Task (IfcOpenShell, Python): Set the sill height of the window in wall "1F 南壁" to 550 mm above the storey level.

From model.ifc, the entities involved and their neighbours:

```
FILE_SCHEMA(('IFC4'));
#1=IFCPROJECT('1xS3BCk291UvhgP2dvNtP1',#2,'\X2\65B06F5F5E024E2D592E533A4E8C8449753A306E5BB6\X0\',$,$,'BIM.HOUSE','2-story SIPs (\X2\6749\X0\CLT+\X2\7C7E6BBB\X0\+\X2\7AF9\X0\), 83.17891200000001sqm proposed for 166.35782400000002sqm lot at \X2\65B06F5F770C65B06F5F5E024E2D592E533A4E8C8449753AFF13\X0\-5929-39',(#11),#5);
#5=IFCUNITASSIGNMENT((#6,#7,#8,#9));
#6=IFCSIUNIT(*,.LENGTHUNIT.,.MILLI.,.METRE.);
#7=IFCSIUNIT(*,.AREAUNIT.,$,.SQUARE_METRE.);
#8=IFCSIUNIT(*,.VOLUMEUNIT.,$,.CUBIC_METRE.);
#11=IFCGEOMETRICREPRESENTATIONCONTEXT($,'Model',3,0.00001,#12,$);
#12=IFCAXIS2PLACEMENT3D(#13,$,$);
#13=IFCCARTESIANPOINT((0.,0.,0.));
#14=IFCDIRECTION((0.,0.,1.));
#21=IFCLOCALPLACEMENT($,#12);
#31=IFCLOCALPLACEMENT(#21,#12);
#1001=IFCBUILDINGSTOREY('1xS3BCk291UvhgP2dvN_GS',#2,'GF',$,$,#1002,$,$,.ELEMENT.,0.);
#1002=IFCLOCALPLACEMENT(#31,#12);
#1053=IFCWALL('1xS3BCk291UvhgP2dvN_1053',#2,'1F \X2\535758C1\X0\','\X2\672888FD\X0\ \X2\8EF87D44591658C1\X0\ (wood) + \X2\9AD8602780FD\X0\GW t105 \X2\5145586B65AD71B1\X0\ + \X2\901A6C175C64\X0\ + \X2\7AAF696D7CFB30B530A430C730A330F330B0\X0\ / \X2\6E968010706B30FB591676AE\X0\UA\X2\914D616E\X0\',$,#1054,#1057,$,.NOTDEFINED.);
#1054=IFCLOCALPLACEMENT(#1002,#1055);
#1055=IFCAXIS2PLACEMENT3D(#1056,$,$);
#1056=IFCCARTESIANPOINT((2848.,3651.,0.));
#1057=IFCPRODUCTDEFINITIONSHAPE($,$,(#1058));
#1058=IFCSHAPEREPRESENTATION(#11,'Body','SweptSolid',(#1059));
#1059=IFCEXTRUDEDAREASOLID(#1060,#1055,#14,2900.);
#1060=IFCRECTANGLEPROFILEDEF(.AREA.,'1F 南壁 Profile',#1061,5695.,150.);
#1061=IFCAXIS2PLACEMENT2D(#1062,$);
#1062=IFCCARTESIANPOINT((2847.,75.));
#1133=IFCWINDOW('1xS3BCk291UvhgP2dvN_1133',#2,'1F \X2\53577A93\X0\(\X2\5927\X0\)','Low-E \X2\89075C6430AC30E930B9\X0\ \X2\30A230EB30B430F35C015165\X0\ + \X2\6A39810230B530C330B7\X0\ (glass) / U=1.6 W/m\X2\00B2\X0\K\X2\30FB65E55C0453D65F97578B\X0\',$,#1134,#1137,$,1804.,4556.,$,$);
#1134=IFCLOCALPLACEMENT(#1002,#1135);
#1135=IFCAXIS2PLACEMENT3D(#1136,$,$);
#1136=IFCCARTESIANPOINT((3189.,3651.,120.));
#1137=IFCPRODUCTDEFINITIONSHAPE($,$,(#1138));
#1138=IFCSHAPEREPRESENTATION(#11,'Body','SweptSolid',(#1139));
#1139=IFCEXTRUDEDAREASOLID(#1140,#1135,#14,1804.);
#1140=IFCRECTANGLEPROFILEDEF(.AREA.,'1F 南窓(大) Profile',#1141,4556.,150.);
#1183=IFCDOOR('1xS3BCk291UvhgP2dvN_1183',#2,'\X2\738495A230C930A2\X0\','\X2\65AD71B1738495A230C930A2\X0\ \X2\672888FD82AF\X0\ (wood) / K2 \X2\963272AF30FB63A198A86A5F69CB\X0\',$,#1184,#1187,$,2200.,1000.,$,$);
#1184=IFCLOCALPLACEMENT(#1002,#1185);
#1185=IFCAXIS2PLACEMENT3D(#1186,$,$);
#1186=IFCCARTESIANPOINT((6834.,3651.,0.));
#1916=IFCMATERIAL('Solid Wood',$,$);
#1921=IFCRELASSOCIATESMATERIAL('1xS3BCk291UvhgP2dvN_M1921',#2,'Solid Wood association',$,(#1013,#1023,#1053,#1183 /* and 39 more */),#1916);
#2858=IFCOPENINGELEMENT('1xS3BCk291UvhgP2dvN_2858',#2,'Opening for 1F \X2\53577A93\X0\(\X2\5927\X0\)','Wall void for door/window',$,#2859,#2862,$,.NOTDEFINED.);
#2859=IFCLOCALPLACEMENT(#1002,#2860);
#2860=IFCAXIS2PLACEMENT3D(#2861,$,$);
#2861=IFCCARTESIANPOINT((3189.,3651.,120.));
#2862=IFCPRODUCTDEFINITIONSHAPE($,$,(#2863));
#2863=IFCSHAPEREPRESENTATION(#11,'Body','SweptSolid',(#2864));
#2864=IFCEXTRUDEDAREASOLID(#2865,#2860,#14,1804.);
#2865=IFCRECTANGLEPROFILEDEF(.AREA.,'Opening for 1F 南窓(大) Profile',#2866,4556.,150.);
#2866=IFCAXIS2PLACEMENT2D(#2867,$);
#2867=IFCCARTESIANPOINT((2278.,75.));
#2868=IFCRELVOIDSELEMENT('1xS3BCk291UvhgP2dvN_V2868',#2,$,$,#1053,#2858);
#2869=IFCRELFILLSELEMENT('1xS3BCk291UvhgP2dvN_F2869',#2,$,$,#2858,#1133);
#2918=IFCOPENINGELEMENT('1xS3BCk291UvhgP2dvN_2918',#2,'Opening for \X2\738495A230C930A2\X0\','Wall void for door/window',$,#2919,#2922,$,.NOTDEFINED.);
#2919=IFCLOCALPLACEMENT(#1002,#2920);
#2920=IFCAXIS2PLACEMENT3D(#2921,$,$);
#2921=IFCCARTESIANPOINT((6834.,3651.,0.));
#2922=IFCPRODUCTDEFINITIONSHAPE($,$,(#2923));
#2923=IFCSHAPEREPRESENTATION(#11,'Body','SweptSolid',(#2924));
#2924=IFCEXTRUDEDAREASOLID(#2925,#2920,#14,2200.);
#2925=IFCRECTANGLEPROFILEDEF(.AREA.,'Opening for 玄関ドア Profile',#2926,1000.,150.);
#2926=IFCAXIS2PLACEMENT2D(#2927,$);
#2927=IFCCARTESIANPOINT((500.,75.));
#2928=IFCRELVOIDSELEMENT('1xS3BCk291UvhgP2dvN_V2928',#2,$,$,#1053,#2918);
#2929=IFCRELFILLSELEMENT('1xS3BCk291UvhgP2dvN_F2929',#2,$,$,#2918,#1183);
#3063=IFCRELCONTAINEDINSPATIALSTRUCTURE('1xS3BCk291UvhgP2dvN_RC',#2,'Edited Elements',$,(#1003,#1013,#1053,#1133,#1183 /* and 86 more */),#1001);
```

```python
import numpy as np
import ifcopenshell
import ifcopenshell.api.geometry
import ifcopenshell.geom
import ifcopenshell.util.element
import ifcopenshell.util.placement
import ifcopenshell.util.shape
import ifcopenshell.util.unit

model = ifcopenshell.open("model.ifc")
unit_scale = ifcopenshell.util.unit.calculate_unit_scale(model)

window = model.by_id(1133)
opening = window.FillsVoids[0].RelatingOpeningElement
storey = ifcopenshell.util.element.get_container(window, ifc_class="IfcBuildingStorey")
level = ifcopenshell.util.placement.get_local_placement(storey.ObjectPlacement)[2, 3]

# The opening's origin need not be at the sill, so measure its lowest point.
shape = ifcopenshell.geom.create_shape(ifcopenshell.geom.settings(), opening)
bottom = ifcopenshell.util.shape.get_shape_bottom_elevation(shape, shape.geometry) / unit_scale
dz = level + 550.0 - bottom

shift = np.array([0.0, 0.0, dz])
# The window is not placed relative to its opening, so move both.
for product in (opening, window):
    matrix = ifcopenshell.util.placement.get_local_placement(product.ObjectPlacement)
    matrix[:3, 3] += shift
    ifcopenshell.api.geometry.edit_object_placement(model, product=product, matrix=matrix, is_si=False)

print(f"moved by {dz * unit_scale:+.3f} m")

model.write("model-out.ifc")
```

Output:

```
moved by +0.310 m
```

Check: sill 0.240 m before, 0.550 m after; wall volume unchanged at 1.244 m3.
